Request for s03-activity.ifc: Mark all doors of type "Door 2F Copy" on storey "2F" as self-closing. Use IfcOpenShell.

First a look at what the model holds.

```python
import ifcopenshell
import ifcopenshell.util.element

model = ifcopenshell.open("s03-activity.ifc")
print(model.schema)
storey = next(s for s in model.by_type("IfcBuildingStorey") if s.Name == "2F")
doors = [e for e in ifcopenshell.util.element.get_decomposition(storey) if e.is_a("IfcDoor")]
seen = {}
for e in doors:
    element_type = ifcopenshell.util.element.get_type(e)
    key = (element_type.Name if element_type != e and element_type else None, ifcopenshell.util.element.get_pset(e, "Pset_DoorCommon", "SelfClosing"))
    seen[key] = seen.get(key, 0) + 1
for (name, value), count in sorted(seen.items(), key=str):
    print(count, "x", name, "|", value)
```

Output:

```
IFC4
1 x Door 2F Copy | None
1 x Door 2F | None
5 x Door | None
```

```python
import ifcopenshell
import ifcopenshell.api.pset
import ifcopenshell.util.element

model = ifcopenshell.open("s03-activity.ifc")

storey = next(s for s in model.by_type("IfcBuildingStorey") if s.Name == "2F")
doors = [e for e in ifcopenshell.util.element.get_decomposition(storey) if e.is_a("IfcDoor")]

count = 0
for e in doors:
    element_type = ifcopenshell.util.element.get_type(e)
    if element_type in (None, e) or element_type.Name != "Door 2F Copy":
        continue
    # add_pset returns the element's existing set when there is one.
    pset = ifcopenshell.api.pset.add_pset(model, product=e, name="Pset_DoorCommon")
    ifcopenshell.api.pset.edit_pset(model, pset=pset, properties={"SelfClosing": True})
    count += 1

print(count, "doors updated")

model.write("s03-activity_updated.ifc")
```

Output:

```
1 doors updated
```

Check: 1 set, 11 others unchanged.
